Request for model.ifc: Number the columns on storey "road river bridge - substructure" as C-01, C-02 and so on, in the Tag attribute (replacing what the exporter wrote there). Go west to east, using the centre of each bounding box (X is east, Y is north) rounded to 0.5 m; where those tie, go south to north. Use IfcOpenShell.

First a look at what the model holds.

```python
import ifcopenshell
import ifcopenshell.util.element
import ifcopenshell.util.placement

model = ifcopenshell.open("model.ifc")
print(model.schema)
storey = next(s for s in model.by_type("IfcBuildingStorey") if s.Name == "road river bridge - substructure")
columns = [e for e in ifcopenshell.util.element.get_decomposition(storey) if e.is_a("IfcColumn")]
for e in sorted(columns, key=lambda e: e.id()):
    origin = ifcopenshell.util.placement.get_local_placement(e.ObjectPlacement)[:3, 3]
    print(e.id(), e.Tag, e.Name, origin.round(2) + 0.0, sep=" | ")
```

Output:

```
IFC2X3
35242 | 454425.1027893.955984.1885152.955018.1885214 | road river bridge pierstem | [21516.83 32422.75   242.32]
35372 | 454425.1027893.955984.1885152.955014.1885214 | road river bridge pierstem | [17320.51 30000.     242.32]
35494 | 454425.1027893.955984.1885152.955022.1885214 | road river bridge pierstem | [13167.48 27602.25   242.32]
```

```python
import ifcopenshell
import ifcopenshell.geom
import ifcopenshell.util.element
import ifcopenshell.util.shape

model = ifcopenshell.open("model.ifc")
settings = ifcopenshell.geom.settings()
settings.set("use-world-coords", True)


def centre(element):
    shape = ifcopenshell.geom.create_shape(settings, element)
    return ifcopenshell.util.shape.get_bbox_centroid(shape.geometry)


storey = next(s for s in model.by_type("IfcBuildingStorey") if s.Name == "road river bridge - substructure")
columns = [e for e in ifcopenshell.util.element.get_decomposition(storey) if e.is_a("IfcColumn")]

# Insertion points can sit at a corner or the storey origin, so sort by the geometry (in metres).
centres = {e: centre(e) for e in columns}
columns.sort(key=lambda e: (round(centres[e][0] / 0.5), centres[e][1]))

for i, e in enumerate(columns, start=1):
    number = f"C-{i:02d}"
    e.Tag = number
    print(e.id(), number)

model.write("model_v2.ifc")
```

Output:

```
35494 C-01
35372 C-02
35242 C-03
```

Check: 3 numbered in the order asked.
